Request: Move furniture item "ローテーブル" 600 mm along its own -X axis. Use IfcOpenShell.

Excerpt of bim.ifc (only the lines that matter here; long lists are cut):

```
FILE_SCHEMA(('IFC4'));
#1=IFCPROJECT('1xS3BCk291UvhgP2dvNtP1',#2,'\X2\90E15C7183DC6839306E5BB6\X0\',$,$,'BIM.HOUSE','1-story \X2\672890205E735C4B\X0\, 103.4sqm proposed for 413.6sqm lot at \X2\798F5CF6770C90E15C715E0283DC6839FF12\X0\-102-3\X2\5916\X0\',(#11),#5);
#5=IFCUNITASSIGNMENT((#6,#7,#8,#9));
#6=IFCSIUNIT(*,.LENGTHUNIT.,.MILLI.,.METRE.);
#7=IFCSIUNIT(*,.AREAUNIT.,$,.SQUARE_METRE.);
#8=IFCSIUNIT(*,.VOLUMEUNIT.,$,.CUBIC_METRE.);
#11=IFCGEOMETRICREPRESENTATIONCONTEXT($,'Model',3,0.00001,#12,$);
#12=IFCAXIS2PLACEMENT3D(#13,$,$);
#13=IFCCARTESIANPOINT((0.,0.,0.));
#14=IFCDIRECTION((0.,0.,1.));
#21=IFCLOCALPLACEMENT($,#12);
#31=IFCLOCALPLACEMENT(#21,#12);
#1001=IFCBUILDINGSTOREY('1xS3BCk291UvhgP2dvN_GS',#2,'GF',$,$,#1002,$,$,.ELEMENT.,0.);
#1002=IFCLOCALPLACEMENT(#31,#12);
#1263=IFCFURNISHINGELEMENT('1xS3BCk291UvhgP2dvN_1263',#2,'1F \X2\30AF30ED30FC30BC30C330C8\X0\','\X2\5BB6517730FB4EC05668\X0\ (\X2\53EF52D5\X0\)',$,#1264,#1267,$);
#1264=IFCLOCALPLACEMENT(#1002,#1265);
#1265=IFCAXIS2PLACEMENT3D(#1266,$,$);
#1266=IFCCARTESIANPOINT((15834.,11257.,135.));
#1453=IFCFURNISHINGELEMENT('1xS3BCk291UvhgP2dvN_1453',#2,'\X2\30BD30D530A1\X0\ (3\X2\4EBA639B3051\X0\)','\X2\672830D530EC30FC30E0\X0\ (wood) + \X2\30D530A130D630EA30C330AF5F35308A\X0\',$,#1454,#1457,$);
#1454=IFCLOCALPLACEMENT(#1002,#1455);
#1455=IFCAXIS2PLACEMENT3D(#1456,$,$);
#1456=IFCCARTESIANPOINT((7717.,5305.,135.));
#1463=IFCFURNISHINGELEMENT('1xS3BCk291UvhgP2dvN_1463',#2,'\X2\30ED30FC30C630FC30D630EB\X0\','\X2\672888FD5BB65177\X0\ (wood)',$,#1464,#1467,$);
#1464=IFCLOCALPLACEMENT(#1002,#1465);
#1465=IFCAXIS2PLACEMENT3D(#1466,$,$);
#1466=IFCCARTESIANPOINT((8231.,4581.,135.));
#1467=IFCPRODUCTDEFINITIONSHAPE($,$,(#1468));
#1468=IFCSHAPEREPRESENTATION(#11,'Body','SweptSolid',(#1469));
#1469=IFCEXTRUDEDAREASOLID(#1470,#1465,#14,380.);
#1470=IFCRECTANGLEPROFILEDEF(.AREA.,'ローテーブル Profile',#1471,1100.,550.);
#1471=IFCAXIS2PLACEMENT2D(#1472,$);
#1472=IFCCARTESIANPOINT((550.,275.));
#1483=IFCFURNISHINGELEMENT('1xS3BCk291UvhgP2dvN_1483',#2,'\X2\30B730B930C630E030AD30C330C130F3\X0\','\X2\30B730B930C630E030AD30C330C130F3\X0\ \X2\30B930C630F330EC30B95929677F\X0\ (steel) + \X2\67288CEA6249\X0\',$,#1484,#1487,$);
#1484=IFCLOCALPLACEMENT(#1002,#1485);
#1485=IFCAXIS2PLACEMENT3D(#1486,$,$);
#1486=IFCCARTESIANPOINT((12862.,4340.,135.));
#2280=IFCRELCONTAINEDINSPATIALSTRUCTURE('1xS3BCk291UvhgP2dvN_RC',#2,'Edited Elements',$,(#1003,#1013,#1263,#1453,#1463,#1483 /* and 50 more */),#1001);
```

```python
import ifcopenshell
import ifcopenshell.api.geometry
import ifcopenshell.util.placement
import ifcopenshell.util.unit

model = ifcopenshell.open("bim.ifc")
unit_scale = ifcopenshell.util.unit.calculate_unit_scale(model)

item = model.by_guid("1xS3BCk291UvhgP2dvN_1463")
matrix = ifcopenshell.util.placement.get_local_placement(item.ObjectPlacement)
matrix[:3, 3] -= matrix[:3, 0] * 0.6 / unit_scale
ifcopenshell.api.geometry.edit_object_placement(model, product=item, matrix=matrix, is_si=False)

print(ifcopenshell.util.placement.get_local_placement(item.ObjectPlacement).round(3) + 0.0)

model.write("bim_rev.ifc")
```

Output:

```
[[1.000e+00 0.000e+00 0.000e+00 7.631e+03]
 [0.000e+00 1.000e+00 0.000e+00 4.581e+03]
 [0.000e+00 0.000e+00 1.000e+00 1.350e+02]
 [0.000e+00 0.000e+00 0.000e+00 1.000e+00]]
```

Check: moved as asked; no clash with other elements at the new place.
